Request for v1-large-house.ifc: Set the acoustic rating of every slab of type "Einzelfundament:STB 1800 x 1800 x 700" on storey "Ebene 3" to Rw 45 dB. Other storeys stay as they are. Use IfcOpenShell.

First a look at what the model holds.

```python
import ifcopenshell
import ifcopenshell.util.element

model = ifcopenshell.open("v1-large-house.ifc")
print(model.schema)
storey = next(s for s in model.by_type("IfcBuildingStorey") if s.Name == "Ebene 3")
slabs = [e for e in ifcopenshell.util.element.get_decomposition(storey) if e.is_a("IfcSlab")]
seen = {}
for e in slabs:
    element_type = ifcopenshell.util.element.get_type(e)
    key = (element_type.Name if element_type != e and element_type else None, ifcopenshell.util.element.get_pset(e, "Pset_SlabCommon", "AcousticRating"))
    seen[key] = seen.get(key, 0) + 1
for (name, value), count in sorted(seen.items(), key=str):
    print(count, "x", name, "|", value)
```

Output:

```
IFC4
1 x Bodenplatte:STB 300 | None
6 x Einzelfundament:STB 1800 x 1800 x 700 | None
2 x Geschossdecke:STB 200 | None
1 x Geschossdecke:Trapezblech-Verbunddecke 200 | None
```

```python
import ifcopenshell
import ifcopenshell.api.pset
import ifcopenshell.util.element

model = ifcopenshell.open("v1-large-house.ifc")

storey = next(s for s in model.by_type("IfcBuildingStorey") if s.Name == "Ebene 3")
slabs = [e for e in ifcopenshell.util.element.get_decomposition(storey) if e.is_a("IfcSlab")]

count = 0
for e in slabs:
    element_type = ifcopenshell.util.element.get_type(e)
    if element_type in (None, e) or element_type.Name != "Einzelfundament:STB 1800 x 1800 x 700":
        continue
    # add_pset returns the element's existing set when there is one.
    pset = ifcopenshell.api.pset.add_pset(model, product=e, name="Pset_SlabCommon")
    ifcopenshell.api.pset.edit_pset(model, pset=pset, properties={"AcousticRating": "Rw 45 dB"})
    count += 1

print(count, "slabs updated")

model.write("v1-large-house_updated.ifc")
```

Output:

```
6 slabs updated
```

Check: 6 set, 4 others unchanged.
